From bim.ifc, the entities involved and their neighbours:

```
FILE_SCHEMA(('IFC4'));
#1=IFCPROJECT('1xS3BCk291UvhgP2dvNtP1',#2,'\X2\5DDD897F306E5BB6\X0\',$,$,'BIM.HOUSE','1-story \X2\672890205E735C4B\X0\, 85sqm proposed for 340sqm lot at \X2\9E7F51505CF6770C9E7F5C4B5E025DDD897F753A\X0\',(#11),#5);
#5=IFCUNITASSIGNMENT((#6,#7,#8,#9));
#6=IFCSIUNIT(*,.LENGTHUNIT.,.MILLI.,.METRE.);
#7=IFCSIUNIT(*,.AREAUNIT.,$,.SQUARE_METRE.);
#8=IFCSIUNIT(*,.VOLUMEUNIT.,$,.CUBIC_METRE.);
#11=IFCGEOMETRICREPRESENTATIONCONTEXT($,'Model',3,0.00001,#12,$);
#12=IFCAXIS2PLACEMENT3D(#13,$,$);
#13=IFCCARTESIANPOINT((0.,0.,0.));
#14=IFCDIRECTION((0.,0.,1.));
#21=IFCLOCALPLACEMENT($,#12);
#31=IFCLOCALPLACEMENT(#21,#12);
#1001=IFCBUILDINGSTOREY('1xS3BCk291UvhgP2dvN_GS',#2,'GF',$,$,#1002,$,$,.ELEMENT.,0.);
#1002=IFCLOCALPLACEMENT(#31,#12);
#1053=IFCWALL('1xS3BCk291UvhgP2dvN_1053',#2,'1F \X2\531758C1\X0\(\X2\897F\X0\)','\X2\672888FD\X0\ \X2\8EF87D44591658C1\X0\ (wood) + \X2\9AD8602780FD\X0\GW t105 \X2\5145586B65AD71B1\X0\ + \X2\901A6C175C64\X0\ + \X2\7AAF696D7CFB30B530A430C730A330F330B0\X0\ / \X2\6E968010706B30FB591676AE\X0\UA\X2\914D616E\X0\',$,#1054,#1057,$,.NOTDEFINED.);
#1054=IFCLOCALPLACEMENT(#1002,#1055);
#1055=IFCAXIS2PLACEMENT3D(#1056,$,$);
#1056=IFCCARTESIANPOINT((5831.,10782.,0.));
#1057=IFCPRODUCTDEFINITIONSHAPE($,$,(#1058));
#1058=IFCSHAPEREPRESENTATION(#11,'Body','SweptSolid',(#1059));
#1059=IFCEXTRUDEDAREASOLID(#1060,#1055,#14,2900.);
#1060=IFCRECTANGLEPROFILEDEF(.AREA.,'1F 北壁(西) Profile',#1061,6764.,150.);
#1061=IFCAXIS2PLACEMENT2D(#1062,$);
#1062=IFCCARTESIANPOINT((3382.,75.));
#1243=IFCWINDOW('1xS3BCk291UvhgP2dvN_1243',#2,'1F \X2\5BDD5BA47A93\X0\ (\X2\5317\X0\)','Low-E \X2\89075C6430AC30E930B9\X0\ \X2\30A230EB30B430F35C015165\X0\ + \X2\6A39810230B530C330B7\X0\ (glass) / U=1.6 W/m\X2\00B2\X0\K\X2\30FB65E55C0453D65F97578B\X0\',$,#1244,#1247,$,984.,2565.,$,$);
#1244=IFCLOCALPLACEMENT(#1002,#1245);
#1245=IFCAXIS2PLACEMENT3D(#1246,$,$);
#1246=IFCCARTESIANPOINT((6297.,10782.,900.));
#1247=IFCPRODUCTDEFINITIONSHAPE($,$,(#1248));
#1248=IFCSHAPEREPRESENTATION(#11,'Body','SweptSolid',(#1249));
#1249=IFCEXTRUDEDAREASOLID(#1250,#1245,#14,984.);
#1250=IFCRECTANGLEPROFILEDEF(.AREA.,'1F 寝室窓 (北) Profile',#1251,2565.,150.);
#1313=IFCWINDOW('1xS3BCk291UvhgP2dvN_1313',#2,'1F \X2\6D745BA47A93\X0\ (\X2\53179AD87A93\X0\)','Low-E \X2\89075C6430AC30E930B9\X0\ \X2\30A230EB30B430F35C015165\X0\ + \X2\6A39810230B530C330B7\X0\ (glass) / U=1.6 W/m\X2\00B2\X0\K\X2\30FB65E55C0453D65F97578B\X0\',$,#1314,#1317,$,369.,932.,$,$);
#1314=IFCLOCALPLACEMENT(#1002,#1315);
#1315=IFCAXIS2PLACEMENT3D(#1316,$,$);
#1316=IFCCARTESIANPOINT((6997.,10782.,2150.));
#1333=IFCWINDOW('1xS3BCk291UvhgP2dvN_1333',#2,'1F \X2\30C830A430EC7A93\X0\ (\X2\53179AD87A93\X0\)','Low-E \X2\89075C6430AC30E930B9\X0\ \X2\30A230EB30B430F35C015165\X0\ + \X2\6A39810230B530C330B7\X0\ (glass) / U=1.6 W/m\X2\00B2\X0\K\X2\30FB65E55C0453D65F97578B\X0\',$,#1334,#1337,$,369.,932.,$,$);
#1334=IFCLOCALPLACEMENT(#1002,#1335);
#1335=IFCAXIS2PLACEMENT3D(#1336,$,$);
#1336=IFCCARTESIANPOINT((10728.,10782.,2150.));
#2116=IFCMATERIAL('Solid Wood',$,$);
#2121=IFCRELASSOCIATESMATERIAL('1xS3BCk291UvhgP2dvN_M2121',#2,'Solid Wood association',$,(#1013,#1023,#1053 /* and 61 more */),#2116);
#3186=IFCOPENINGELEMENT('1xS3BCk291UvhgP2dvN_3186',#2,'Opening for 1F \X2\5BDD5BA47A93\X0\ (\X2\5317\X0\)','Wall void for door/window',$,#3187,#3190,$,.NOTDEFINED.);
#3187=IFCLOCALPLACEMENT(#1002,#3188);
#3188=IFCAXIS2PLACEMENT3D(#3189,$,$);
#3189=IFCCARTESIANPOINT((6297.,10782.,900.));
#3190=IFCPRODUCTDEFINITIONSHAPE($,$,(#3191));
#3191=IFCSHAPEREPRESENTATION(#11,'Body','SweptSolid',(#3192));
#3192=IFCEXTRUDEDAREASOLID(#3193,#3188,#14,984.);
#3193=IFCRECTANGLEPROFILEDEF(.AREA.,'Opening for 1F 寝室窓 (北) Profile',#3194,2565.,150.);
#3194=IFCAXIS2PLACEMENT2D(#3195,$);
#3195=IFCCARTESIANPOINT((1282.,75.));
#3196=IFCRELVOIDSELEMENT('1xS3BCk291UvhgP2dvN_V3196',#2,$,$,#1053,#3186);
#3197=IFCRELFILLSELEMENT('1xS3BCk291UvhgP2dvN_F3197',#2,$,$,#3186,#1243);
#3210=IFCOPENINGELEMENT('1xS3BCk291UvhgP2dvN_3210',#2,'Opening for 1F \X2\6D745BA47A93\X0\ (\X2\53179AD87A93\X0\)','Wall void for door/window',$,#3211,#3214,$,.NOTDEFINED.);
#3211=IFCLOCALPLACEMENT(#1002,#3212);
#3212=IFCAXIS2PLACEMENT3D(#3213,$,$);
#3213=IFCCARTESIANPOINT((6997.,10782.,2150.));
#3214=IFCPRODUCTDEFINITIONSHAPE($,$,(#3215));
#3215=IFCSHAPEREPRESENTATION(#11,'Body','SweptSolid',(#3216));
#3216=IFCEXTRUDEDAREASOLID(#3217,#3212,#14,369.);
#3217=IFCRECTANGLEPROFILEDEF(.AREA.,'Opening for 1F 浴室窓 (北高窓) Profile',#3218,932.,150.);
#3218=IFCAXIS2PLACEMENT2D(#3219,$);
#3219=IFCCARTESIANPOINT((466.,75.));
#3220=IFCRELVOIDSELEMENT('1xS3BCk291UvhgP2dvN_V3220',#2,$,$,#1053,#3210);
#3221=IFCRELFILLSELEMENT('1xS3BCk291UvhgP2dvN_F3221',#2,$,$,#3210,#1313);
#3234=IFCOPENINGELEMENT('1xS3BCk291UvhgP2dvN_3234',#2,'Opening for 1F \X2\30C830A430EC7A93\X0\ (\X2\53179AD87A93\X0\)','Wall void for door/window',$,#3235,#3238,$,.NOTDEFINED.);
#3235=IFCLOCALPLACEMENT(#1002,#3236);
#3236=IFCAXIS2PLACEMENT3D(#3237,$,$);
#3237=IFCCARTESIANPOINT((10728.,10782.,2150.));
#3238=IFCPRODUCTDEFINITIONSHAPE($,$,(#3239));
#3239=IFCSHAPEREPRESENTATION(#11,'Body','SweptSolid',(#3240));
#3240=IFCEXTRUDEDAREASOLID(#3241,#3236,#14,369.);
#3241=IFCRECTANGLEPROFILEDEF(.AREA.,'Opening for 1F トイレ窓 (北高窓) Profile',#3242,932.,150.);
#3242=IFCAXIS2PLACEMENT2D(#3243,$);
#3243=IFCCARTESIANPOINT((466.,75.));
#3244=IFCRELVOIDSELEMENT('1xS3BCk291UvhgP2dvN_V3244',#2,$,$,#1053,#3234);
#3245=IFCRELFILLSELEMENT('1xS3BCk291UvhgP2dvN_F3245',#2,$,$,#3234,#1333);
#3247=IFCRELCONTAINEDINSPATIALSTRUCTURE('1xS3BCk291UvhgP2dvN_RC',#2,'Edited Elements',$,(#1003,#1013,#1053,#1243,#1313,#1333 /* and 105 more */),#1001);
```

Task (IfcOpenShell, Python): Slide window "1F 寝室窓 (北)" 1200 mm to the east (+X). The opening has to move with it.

```python
import ifcopenshell
import ifcopenshell.api.geometry
import ifcopenshell.util.placement

model = ifcopenshell.open("bim.ifc")

window = model.by_guid("1xS3BCk291UvhgP2dvN_1243")
opening = window.FillsVoids[0].RelatingOpeningElement
wall = opening.VoidsElements[0].RelatingBuildingElement

wall_matrix = ifcopenshell.util.placement.get_local_placement(wall.ObjectPlacement)
shift = wall_matrix[:3, 0] * 1200.0
before = ifcopenshell.util.placement.get_local_placement(window.ObjectPlacement)[:3, 3].copy()

# The window is not placed relative to its opening, so move both.
for product in (opening, window):
    matrix = ifcopenshell.util.placement.get_local_placement(product.ObjectPlacement)
    matrix[:3, 3] += shift
    ifcopenshell.api.geometry.edit_object_placement(model, product=product, matrix=matrix, is_si=False)

after = ifcopenshell.util.placement.get_local_placement(window.ObjectPlacement)[:3, 3]
print("window moved by", (after - before).round(3) + 0.0)

model.write("bim_updated.ifc")
```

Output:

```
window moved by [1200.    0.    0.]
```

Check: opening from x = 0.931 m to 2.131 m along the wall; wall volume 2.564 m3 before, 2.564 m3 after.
